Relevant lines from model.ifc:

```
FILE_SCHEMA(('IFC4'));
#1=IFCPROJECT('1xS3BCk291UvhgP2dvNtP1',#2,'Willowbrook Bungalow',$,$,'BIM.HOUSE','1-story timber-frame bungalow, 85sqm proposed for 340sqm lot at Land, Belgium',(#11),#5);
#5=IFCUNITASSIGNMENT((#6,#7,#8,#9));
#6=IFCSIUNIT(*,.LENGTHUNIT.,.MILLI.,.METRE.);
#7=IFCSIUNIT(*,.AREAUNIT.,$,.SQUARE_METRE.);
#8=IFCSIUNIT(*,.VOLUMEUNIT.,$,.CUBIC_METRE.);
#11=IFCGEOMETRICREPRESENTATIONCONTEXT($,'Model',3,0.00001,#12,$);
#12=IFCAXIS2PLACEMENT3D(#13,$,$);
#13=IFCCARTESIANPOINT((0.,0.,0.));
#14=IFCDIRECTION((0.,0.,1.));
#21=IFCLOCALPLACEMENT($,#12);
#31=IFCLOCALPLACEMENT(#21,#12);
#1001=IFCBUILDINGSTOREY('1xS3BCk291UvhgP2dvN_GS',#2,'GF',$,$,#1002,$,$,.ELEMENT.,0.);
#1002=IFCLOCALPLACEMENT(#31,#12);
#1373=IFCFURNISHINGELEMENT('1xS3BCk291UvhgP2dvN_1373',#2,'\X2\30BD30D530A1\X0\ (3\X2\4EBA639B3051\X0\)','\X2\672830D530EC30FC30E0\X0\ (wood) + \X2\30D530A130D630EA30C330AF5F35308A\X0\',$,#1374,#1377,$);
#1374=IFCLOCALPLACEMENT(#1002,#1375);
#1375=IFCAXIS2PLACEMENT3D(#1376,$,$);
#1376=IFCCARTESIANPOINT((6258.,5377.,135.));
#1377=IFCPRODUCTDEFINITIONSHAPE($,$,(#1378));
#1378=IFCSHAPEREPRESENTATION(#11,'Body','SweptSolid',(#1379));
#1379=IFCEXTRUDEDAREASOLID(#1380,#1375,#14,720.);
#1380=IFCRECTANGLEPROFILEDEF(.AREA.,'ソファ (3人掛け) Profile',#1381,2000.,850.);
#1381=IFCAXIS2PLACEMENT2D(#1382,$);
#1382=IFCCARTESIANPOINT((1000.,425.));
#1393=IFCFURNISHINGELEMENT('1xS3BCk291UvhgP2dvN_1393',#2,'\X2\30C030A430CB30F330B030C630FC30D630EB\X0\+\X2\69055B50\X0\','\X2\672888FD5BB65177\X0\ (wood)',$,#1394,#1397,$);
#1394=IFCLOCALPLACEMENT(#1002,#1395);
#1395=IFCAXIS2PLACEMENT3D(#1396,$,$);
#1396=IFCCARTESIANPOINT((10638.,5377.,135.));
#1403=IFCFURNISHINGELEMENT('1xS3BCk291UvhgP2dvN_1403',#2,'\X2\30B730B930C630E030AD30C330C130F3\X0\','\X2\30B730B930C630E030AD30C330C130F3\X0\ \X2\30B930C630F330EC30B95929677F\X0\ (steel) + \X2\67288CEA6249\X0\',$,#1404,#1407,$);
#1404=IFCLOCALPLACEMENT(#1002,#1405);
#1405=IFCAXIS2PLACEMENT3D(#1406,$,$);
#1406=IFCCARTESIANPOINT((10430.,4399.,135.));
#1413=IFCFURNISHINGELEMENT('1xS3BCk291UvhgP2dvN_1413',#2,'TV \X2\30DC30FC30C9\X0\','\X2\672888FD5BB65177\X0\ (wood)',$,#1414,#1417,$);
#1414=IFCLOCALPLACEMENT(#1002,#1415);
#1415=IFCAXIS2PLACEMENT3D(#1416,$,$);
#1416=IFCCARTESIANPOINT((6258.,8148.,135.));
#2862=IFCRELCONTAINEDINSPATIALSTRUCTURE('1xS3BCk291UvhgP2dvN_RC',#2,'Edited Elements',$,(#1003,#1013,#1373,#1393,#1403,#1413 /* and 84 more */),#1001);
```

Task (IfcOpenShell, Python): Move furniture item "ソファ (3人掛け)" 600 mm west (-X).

```python
import ifcopenshell
import ifcopenshell.api.geometry
import ifcopenshell.util.placement
import ifcopenshell.util.unit

model = ifcopenshell.open("model.ifc")
unit_scale = ifcopenshell.util.unit.calculate_unit_scale(model)

item = model.by_guid("1xS3BCk291UvhgP2dvN_1373")
matrix = ifcopenshell.util.placement.get_local_placement(item.ObjectPlacement)
matrix[0, 3] -= 0.6 / unit_scale
ifcopenshell.api.geometry.edit_object_placement(model, product=item, matrix=matrix, is_si=False)

print(ifcopenshell.util.placement.get_local_placement(item.ObjectPlacement).round(3) + 0.0)

model.write("model_edited.ifc")
```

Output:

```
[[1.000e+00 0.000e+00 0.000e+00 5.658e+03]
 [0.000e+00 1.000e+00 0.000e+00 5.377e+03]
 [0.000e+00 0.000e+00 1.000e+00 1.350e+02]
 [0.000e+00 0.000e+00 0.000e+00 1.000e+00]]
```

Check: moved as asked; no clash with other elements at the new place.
